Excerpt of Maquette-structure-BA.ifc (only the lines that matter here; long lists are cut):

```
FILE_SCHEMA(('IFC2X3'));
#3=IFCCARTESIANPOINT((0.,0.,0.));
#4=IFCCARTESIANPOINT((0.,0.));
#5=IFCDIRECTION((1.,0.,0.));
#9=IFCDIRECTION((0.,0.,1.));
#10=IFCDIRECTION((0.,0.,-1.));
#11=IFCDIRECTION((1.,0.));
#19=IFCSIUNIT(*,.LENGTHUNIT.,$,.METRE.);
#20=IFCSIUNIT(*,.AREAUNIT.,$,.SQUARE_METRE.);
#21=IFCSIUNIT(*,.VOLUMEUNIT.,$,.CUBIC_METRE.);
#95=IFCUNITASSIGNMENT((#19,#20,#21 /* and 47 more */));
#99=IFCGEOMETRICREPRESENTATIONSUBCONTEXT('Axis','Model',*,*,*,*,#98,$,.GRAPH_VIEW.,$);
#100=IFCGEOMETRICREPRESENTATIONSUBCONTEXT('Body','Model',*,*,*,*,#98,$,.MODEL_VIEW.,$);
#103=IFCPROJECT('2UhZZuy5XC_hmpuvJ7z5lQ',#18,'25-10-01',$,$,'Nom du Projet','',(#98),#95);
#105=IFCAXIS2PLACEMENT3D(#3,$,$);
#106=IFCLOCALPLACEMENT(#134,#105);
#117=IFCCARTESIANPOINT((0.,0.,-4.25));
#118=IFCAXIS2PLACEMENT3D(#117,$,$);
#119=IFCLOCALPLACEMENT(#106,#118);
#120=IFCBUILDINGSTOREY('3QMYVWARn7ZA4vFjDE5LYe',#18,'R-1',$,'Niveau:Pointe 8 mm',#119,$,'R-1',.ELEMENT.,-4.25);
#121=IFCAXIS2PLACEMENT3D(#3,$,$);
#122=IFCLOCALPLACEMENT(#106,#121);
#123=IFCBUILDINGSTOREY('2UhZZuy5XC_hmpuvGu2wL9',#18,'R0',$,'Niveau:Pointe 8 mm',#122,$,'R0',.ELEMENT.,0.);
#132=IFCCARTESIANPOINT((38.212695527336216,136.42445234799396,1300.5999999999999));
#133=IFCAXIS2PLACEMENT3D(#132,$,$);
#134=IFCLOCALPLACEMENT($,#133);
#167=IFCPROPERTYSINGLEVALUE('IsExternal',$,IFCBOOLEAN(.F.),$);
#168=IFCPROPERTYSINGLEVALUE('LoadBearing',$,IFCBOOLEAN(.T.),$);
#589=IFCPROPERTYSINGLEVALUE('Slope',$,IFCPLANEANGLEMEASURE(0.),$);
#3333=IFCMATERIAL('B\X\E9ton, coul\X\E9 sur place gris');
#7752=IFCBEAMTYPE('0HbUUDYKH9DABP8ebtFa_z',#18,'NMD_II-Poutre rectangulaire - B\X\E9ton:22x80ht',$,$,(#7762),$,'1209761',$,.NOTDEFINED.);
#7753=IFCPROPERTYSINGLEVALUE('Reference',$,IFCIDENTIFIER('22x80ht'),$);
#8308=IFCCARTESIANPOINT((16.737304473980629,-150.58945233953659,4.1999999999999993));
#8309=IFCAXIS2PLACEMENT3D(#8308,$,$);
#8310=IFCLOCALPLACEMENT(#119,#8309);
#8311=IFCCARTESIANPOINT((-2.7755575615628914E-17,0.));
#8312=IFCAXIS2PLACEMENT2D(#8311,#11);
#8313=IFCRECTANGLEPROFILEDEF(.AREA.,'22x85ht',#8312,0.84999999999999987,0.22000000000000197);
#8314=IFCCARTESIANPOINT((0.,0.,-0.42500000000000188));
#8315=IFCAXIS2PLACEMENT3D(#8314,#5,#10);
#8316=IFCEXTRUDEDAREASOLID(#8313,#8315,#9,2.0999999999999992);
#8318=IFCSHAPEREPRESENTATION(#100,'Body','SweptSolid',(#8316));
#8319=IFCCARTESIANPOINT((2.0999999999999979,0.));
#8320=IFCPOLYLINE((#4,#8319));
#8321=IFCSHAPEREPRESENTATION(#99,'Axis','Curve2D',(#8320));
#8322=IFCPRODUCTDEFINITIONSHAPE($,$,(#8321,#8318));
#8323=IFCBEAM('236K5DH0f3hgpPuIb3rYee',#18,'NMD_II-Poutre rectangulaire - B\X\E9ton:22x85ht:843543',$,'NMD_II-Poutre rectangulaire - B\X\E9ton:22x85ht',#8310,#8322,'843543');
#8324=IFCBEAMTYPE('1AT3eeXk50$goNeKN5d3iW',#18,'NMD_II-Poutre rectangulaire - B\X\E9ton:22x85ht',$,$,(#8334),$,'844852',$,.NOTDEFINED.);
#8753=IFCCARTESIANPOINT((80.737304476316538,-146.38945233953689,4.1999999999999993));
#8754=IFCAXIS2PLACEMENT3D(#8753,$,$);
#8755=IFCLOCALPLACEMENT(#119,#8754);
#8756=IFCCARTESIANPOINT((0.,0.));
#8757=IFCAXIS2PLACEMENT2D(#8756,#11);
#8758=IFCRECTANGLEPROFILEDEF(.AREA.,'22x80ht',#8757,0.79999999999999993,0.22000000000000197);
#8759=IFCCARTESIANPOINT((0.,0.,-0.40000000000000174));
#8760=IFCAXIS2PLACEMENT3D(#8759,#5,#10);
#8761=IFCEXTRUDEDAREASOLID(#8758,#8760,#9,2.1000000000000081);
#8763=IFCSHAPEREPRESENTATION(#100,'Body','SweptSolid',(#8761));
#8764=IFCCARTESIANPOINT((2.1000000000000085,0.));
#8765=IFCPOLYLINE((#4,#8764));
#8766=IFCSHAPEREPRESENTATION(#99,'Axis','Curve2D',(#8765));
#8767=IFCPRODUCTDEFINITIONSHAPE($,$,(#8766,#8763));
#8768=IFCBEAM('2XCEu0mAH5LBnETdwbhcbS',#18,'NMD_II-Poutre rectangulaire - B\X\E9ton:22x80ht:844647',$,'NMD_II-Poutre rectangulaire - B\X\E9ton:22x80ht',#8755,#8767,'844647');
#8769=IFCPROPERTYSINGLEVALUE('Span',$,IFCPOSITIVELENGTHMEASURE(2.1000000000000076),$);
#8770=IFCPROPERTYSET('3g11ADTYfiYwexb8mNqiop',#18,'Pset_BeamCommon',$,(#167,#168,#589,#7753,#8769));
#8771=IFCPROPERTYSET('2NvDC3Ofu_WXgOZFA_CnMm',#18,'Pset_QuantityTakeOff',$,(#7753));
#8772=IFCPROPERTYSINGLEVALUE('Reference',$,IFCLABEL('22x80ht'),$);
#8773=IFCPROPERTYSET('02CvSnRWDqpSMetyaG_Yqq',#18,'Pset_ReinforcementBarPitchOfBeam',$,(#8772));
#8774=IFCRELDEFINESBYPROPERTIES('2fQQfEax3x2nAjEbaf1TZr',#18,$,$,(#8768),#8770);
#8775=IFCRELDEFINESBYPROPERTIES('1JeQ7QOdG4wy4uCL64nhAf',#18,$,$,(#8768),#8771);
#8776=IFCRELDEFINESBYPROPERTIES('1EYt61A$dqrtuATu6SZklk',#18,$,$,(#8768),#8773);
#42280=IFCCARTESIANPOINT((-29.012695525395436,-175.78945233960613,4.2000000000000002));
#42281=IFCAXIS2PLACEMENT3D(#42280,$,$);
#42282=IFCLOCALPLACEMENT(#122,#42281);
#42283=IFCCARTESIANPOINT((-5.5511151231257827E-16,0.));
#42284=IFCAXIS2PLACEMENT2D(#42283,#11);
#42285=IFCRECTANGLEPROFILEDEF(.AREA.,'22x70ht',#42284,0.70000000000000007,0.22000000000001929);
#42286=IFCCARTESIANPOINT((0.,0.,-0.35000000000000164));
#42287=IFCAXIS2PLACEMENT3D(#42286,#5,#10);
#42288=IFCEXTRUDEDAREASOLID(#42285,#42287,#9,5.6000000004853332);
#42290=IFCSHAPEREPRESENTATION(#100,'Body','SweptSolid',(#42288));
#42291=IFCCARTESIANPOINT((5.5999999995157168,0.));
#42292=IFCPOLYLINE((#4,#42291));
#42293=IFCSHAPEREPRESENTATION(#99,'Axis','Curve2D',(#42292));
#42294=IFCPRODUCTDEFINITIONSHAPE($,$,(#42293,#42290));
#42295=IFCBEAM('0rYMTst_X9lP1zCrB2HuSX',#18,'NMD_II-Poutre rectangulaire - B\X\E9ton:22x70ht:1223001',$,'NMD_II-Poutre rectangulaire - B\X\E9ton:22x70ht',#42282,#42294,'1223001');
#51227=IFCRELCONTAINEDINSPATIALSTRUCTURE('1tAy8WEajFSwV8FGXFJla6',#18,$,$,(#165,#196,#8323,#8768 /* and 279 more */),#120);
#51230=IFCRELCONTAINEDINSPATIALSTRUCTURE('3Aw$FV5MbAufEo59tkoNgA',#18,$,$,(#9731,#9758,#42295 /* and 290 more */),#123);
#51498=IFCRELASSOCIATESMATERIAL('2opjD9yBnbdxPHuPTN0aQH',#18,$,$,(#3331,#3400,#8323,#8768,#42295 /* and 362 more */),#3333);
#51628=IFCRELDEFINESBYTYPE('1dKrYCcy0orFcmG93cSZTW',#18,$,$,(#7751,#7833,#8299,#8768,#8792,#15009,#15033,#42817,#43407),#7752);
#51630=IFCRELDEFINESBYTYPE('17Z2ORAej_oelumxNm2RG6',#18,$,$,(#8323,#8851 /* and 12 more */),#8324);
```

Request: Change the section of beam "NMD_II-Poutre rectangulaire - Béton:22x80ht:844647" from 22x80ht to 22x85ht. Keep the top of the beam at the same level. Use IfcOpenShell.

```python
import ifcopenshell
import ifcopenshell.api.pset
import ifcopenshell.api.type
import ifcopenshell.util.element
import ifcopenshell.util.representation

model = ifcopenshell.open("Maquette-structure-BA.ifc")

member = model.by_guid("2XCEu0mAH5LBnETdwbhcbS")
source = next(p for p in model.by_type("IfcRectangleProfileDef") if p.ProfileName == "22x85ht")

body = ifcopenshell.util.representation.get_representation(member, "Model", "Body")
solid = body.Items[0]
old_profile = solid.SweptArea

# Copy the section's sizes but keep this member's own profile position.
profile = ifcopenshell.util.element.copy(model, source)
# Profiles are centred, so shift by half the change in depth to hold the top.
shift = (old_profile.XDim - profile.XDim) / 2
x, y = old_profile.Position.Location.Coordinates
up = (-1.0, 0.0)  # upwards, in the solid's own plane
location = model.createIfcCartesianPoint((x + up[0] * shift, y + up[1] * shift))
profile.Position = model.createIfcAxis2Placement2D(location, old_profile.Position.RefDirection)
solid.SweptArea = profile
if not model.get_total_inverses(old_profile):
    ifcopenshell.util.element.remove_deep2(model, old_profile)

new_type = model.by_id(8324)
ifcopenshell.api.type.assign_type(
    model, related_objects=[member], relating_type=new_type, should_map_representations=False
)
member.Name = member.Name.replace("22x80ht", "22x85ht")
member.ObjectType = "NMD_II-Poutre rectangulaire - Béton:22x85ht"
pset = model.by_id(ifcopenshell.util.element.get_pset(member, "Pset_BeamCommon", should_inherit=False)["id"])
ifcopenshell.api.pset.edit_pset(model, pset=pset, properties={"Reference": "22x85ht"})
pset = model.by_id(ifcopenshell.util.element.get_pset(member, "Pset_QuantityTakeOff", should_inherit=False)["id"])
ifcopenshell.api.pset.edit_pset(model, pset=pset, properties={"Reference": "22x85ht"})
pset = model.by_id(ifcopenshell.util.element.get_pset(member, "Pset_ReinforcementBarPitchOfBeam", should_inherit=False)["id"])
ifcopenshell.api.pset.edit_pset(model, pset=pset, properties={"Reference": "22x85ht"})

print(solid.SweptArea)

model.write("Maquette-structure-BA-out.ifc")
```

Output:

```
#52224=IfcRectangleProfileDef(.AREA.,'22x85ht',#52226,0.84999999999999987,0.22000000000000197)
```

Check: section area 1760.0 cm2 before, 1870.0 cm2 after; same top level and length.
